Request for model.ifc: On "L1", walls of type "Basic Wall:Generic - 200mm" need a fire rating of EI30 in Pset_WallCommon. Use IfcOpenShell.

First a look at what the model holds.

```python
import ifcopenshell
import ifcopenshell.util.element

model = ifcopenshell.open("model.ifc")
print(model.schema)
storey = next(s for s in model.by_type("IfcBuildingStorey") if s.Name == "L1")
walls = [e for e in ifcopenshell.util.element.get_decomposition(storey) if e.is_a("IfcWall")]
seen = {}
for e in walls:
    element_type = ifcopenshell.util.element.get_type(e)
    key = (element_type.Name if element_type != e and element_type else None, ifcopenshell.util.element.get_pset(e, "Pset_WallCommon", "FireRating"))
    seen[key] = seen.get(key, 0) + 1
for (name, value), count in sorted(seen.items(), key=str):
    print(count, "x", name, "|", value)
```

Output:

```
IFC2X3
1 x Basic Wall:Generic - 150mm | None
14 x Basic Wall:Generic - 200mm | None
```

```python
import ifcopenshell
import ifcopenshell.api.pset
import ifcopenshell.util.element

model = ifcopenshell.open("model.ifc")

storey = next(s for s in model.by_type("IfcBuildingStorey") if s.Name == "L1")
walls = [e for e in ifcopenshell.util.element.get_decomposition(storey) if e.is_a("IfcWall")]

count = 0
for e in walls:
    element_type = ifcopenshell.util.element.get_type(e)
    if element_type in (None, e) or element_type.Name != "Basic Wall:Generic - 200mm":
        continue
    # add_pset returns the element's existing set when there is one.
    pset = ifcopenshell.api.pset.add_pset(model, product=e, name="Pset_WallCommon")
    ifcopenshell.api.pset.edit_pset(model, pset=pset, properties={"FireRating": "EI30"})
    count += 1

print(count, "walls updated")

model.write("model_v2.ifc")
```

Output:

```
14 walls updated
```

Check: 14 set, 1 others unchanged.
